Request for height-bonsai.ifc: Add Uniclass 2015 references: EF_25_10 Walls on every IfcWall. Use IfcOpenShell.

First a look at what the model holds.

```python
import ifcopenshell

model = ifcopenshell.open("height-bonsai.ifc")
print(model.schema)
print("classifications:", [c.Name for c in model.by_type("IfcClassification")])
for ifc_class in ("IfcDoor", "IfcRoof", "IfcStair", "IfcWall", "IfcWindow"):
    print(ifc_class, len(model.by_type(ifc_class)))
```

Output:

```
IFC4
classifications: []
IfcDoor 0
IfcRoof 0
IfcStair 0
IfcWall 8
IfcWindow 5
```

```python
import ifcopenshell
import ifcopenshell.api.classification

model = ifcopenshell.open("height-bonsai.ifc")

system = ifcopenshell.api.classification.add_classification(model, classification="Uniclass 2015")

codes = {
    "IfcWall": ("EF_25_10", "Walls"),
}
for ifc_class, (code, name) in codes.items():
    products = model.by_type(ifc_class)
    ifcopenshell.api.classification.add_reference(
        model, products=products, classification=system, identification=code, name=name
    )
    print(code, len(products))

model.write("height-bonsai_updated.ifc")
```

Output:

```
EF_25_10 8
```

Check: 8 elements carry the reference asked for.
